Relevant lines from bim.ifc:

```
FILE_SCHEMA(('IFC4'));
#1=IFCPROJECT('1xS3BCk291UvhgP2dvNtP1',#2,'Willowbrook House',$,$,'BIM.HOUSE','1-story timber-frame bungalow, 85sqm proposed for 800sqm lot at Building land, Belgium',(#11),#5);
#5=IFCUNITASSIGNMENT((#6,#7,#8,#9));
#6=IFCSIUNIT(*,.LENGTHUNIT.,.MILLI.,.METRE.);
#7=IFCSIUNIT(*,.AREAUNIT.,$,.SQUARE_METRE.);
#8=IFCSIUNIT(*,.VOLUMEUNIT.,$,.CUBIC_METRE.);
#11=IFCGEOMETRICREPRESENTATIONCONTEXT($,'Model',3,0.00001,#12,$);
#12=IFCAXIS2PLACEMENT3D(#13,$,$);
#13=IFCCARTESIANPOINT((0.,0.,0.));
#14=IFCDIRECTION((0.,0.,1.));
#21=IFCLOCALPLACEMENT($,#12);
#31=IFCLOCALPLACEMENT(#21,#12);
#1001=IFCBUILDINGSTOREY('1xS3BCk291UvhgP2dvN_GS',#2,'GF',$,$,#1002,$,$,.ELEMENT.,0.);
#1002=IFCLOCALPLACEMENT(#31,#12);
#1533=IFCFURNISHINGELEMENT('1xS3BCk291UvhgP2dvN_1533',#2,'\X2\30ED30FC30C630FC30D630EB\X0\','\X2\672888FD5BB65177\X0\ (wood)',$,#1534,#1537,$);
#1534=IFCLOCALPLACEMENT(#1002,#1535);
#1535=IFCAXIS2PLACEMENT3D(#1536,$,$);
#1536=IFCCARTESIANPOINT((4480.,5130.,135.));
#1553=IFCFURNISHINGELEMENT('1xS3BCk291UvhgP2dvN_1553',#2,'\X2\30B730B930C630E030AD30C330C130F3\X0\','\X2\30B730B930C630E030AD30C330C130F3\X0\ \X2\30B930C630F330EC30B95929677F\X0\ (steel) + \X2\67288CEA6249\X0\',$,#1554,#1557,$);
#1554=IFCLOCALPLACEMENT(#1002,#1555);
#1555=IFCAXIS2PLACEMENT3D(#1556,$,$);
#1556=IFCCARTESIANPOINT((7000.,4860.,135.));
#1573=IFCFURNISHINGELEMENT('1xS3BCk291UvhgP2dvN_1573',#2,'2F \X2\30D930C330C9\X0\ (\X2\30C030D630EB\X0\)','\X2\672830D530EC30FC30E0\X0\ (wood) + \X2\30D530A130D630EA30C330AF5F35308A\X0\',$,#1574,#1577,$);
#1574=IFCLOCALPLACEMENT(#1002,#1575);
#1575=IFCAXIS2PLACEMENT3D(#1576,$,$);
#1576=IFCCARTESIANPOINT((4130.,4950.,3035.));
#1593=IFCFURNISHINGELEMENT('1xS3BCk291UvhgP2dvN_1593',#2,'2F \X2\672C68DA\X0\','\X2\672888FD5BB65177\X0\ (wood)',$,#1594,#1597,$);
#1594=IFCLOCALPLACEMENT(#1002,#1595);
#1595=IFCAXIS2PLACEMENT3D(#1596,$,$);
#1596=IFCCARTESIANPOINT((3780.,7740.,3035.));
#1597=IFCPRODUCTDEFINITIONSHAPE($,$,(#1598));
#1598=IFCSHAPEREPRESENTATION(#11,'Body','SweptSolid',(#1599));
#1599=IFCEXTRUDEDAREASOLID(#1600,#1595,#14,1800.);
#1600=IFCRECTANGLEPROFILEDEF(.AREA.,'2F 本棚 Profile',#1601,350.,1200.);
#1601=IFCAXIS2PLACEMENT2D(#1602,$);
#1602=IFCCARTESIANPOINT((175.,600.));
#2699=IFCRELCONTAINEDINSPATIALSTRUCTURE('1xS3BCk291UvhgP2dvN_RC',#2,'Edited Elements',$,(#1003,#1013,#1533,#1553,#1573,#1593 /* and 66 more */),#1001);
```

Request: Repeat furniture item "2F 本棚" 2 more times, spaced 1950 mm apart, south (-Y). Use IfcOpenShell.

```python
import numpy as np
import ifcopenshell
import ifcopenshell.api.geometry
import ifcopenshell.api.root
import ifcopenshell.util.element
import ifcopenshell.util.placement
import ifcopenshell.util.unit

model = ifcopenshell.open("bim.ifc")
unit_scale = ifcopenshell.util.unit.calculate_unit_scale(model)


def reuse_history(source, copy):
    """copy_class also copies each property set's owner history, people and application; keep the originals."""
    for rel in copy.IsDefinedBy:
        if rel.is_a("IfcRelDefinesByProperties") and (history := rel.RelatingPropertyDefinition.OwnerHistory):
            rel.RelatingPropertyDefinition.OwnerHistory = source.OwnerHistory
            ifcopenshell.util.element.remove_deep2(model, history)


source = model.by_id(1593)
base = ifcopenshell.util.placement.get_local_placement(source.ObjectPlacement)
step = np.array([0.0, -1.0, 0.0]) * 1.95 / unit_scale

for i in range(1, 3):
    copy = ifcopenshell.api.root.copy_class(model, product=source)
    copy.Representation = ifcopenshell.util.element.copy_deep(
        model, source.Representation, exclude=["IfcGeometricRepresentationContext", "IfcRepresentationMap"]
    )
    reuse_history(source, copy)
    matrix = base.copy()
    matrix[:3, 3] += i * step
    print("added at", matrix[:3, 3].round(3) + 0.0)
    ifcopenshell.api.geometry.edit_object_placement(model, product=copy, matrix=matrix, is_si=False)

model.write("bim_updated.ifc")
```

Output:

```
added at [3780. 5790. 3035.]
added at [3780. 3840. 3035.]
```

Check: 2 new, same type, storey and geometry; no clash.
